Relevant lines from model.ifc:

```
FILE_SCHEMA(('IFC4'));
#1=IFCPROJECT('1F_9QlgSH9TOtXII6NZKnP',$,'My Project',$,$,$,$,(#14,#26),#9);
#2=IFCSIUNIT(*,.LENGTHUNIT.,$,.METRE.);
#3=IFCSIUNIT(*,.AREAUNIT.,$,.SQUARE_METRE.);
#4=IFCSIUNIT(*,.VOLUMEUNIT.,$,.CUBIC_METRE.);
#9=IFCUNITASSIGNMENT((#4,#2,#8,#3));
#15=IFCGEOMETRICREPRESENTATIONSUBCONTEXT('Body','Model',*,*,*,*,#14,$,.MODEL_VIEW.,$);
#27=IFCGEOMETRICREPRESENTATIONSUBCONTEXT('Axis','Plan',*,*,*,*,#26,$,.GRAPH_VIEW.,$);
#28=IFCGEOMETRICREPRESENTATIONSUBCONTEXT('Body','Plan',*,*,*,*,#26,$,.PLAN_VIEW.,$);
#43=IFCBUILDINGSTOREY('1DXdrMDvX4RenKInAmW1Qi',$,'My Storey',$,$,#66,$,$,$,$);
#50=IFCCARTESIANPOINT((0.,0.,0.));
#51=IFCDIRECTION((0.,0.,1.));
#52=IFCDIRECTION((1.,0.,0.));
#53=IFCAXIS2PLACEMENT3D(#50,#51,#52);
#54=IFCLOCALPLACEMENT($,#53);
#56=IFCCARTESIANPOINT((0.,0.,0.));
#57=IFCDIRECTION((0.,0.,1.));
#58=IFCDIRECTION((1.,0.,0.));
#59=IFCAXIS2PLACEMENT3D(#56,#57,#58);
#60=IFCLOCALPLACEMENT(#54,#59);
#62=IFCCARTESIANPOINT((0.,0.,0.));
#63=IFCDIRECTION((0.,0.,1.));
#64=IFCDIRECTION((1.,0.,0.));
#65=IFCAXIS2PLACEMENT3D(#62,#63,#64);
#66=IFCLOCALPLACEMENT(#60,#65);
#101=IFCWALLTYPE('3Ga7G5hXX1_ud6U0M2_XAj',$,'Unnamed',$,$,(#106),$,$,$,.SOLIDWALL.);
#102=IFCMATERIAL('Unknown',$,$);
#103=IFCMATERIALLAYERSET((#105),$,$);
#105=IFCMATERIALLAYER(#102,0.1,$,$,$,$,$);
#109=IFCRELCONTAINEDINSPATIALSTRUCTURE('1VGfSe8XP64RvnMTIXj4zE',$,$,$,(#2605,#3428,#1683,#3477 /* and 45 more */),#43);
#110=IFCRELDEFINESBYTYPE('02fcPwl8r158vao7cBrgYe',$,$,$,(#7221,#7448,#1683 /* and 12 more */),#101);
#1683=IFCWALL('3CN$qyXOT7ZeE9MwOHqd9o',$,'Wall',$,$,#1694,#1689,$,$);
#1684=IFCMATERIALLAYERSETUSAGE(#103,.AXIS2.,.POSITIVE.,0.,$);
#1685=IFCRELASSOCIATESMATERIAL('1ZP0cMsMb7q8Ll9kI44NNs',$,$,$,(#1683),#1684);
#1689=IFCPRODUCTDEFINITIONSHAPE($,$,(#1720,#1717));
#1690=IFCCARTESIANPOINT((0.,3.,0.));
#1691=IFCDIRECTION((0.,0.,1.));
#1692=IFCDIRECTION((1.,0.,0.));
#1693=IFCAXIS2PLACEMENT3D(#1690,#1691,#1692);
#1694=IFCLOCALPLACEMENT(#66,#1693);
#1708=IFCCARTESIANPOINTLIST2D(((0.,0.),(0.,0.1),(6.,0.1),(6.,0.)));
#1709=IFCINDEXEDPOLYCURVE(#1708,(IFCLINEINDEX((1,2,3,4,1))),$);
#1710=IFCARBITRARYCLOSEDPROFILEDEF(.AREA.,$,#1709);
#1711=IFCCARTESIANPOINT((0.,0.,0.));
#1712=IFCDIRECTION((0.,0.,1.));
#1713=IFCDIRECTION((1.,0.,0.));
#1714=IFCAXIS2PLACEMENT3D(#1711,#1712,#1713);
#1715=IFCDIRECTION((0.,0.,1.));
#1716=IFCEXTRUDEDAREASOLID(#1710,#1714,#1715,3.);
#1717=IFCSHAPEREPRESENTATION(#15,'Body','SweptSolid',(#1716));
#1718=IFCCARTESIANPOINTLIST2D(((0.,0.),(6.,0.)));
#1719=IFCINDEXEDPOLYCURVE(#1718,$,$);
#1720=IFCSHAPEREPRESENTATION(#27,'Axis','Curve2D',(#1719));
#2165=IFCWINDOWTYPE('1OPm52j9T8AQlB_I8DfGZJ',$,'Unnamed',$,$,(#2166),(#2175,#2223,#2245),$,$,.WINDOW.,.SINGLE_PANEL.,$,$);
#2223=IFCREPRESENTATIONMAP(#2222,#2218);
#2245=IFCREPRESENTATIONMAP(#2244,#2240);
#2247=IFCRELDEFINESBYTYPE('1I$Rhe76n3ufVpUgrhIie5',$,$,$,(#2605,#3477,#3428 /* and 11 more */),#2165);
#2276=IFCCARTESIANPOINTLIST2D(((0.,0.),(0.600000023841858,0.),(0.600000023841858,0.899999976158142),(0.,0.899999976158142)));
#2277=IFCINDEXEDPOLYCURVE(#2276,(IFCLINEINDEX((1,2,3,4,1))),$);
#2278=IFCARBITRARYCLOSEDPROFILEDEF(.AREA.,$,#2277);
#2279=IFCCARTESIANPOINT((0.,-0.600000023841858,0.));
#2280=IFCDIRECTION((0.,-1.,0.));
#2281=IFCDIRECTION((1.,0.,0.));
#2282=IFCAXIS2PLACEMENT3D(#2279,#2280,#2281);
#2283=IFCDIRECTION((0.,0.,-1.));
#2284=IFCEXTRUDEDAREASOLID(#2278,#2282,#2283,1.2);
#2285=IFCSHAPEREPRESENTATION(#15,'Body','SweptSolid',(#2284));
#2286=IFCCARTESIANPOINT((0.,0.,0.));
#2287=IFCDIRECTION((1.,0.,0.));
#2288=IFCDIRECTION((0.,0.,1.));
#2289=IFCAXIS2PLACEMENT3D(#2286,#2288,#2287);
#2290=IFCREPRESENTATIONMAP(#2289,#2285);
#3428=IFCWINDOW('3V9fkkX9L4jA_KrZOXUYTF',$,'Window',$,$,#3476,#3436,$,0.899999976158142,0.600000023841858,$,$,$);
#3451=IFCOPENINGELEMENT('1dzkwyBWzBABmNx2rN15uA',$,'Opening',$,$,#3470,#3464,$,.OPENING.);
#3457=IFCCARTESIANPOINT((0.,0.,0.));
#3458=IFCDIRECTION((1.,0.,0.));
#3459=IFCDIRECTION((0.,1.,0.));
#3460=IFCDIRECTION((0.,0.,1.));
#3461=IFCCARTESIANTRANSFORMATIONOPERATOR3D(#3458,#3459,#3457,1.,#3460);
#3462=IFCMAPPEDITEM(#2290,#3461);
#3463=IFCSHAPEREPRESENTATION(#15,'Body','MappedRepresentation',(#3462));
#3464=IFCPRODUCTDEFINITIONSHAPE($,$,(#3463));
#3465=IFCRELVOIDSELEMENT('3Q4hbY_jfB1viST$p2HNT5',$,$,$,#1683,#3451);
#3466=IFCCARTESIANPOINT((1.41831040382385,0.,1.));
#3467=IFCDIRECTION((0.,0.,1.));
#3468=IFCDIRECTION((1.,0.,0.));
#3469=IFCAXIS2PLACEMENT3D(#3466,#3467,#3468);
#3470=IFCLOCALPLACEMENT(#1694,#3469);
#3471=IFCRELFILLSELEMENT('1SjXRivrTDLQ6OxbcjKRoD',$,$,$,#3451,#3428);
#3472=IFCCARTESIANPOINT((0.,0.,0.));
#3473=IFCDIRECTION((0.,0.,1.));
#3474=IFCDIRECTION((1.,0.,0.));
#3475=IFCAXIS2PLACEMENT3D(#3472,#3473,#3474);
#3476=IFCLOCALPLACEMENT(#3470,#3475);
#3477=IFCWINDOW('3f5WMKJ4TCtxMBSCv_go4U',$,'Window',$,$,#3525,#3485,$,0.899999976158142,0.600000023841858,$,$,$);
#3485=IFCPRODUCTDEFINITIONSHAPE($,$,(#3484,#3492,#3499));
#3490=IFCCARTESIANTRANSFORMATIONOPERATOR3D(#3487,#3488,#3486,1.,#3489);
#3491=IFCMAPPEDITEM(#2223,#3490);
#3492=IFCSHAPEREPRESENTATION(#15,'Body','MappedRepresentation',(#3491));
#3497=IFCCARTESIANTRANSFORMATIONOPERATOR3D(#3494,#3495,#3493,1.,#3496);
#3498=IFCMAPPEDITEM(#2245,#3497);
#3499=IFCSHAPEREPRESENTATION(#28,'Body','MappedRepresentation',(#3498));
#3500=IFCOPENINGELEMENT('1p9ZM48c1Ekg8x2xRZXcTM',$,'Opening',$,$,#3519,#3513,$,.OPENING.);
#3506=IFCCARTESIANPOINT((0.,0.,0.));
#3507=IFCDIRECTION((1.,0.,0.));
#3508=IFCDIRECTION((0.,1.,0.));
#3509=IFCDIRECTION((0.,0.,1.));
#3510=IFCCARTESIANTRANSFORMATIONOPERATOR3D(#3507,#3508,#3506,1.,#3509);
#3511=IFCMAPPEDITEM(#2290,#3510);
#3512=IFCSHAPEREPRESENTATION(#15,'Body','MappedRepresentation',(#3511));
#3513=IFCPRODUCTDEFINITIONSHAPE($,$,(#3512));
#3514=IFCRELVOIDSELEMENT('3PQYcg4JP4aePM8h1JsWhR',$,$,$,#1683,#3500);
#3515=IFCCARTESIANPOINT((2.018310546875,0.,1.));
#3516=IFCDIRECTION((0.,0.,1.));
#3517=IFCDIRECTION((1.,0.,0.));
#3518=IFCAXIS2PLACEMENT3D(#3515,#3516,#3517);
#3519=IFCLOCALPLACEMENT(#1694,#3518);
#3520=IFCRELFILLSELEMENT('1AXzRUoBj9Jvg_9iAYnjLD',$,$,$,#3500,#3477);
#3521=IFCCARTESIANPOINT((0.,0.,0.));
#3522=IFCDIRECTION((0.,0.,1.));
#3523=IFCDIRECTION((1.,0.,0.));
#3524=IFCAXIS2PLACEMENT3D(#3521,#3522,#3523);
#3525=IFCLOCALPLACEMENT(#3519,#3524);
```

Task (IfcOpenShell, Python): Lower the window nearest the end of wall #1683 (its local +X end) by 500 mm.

```python
import numpy as np
import ifcopenshell
import ifcopenshell.api.geometry
import ifcopenshell.util.placement
import ifcopenshell.util.unit

model = ifcopenshell.open("model.ifc")
unit_scale = ifcopenshell.util.unit.calculate_unit_scale(model)

window = model.by_guid("3f5WMKJ4TCtxMBSCv_go4U")
opening = window.FillsVoids[0].RelatingOpeningElement
dz = -0.5

shift = np.array([0.0, 0.0, dz])
# The window is placed relative to its opening, so it follows when the opening moves.
matrix = ifcopenshell.util.placement.get_local_placement(opening.ObjectPlacement)
matrix[:3, 3] += shift
ifcopenshell.api.geometry.edit_object_placement(
    model, product=opening, matrix=matrix, is_si=False, should_transform_children=True
)

print(f"moved by {dz * unit_scale:+.3f} m")

model.write("model_rev.ifc")
```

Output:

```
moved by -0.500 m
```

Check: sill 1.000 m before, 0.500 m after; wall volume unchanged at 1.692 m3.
